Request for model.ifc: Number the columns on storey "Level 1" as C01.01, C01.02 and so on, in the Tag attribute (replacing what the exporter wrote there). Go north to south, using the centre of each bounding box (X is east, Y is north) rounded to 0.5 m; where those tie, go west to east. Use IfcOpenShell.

First a look at what the model holds.

```python
import ifcopenshell
import ifcopenshell.util.element
import ifcopenshell.util.placement

model = ifcopenshell.open("model.ifc")
print(model.schema)
storey = next(s for s in model.by_type("IfcBuildingStorey") if s.Name == "Level 1")
columns = [e for e in ifcopenshell.util.element.get_decomposition(storey) if e.is_a("IfcColumn")]
for e in sorted(columns, key=lambda e: e.id()):
    origin = ifcopenshell.util.placement.get_local_placement(e.ObjectPlacement)[:3, 3]
    print(e.id(), e.Tag, e.Name, origin.round(2) + 0.0, sep=" | ")
```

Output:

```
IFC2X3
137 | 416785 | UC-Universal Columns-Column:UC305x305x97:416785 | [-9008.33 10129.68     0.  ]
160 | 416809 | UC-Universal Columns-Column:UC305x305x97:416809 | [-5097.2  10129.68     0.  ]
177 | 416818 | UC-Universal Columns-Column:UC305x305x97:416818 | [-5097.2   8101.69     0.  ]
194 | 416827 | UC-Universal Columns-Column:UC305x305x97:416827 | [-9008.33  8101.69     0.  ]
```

```python
import ifcopenshell
import ifcopenshell.geom
import ifcopenshell.util.element
import ifcopenshell.util.shape

model = ifcopenshell.open("model.ifc")
settings = ifcopenshell.geom.settings()
settings.set("use-world-coords", True)


def centre(element):
    shape = ifcopenshell.geom.create_shape(settings, element)
    return ifcopenshell.util.shape.get_bbox_centroid(shape.geometry)


storey = next(s for s in model.by_type("IfcBuildingStorey") if s.Name == "Level 1")
columns = [e for e in ifcopenshell.util.element.get_decomposition(storey) if e.is_a("IfcColumn")]

# Insertion points can sit at a corner or the storey origin, so sort by the geometry (in metres).
centres = {e: centre(e) for e in columns}
columns.sort(key=lambda e: (-round(centres[e][1] / 0.5), centres[e][0]))

for i, e in enumerate(columns, start=1):
    number = f"C01.{i:02d}"
    e.Tag = number
    print(e.id(), number)

model.write("model-out.ifc")
```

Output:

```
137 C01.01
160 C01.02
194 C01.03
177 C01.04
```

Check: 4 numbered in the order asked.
